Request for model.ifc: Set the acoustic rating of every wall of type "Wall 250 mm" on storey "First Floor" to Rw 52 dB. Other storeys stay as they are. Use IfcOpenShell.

First a look at what the model holds.

```python
import ifcopenshell
import ifcopenshell.util.element

model = ifcopenshell.open("model.ifc")
print(model.schema)
storey = next(s for s in model.by_type("IfcBuildingStorey") if s.Name == "First Floor")
walls = [e for e in ifcopenshell.util.element.get_decomposition(storey) if e.is_a("IfcWall")]
seen = {}
for e in walls:
    element_type = ifcopenshell.util.element.get_type(e)
    key = (element_type.Name if element_type != e and element_type else None, ifcopenshell.util.element.get_pset(e, "Pset_WallCommon", "AcousticRating"))
    seen[key] = seen.get(key, 0) + 1
for (name, value), count in sorted(seen.items(), key=str):
    print(count, "x", name, "|", value)
```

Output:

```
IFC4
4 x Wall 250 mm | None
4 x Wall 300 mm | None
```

```python
import ifcopenshell
import ifcopenshell.api.pset
import ifcopenshell.util.element

model = ifcopenshell.open("model.ifc")

storey = next(s for s in model.by_type("IfcBuildingStorey") if s.Name == "First Floor")
walls = [e for e in ifcopenshell.util.element.get_decomposition(storey) if e.is_a("IfcWall")]

count = 0
for e in walls:
    element_type = ifcopenshell.util.element.get_type(e)
    if element_type in (None, e) or element_type.Name != "Wall 250 mm":
        continue
    # add_pset returns the element's existing set when there is one.
    pset = ifcopenshell.api.pset.add_pset(model, product=e, name="Pset_WallCommon")
    ifcopenshell.api.pset.edit_pset(model, pset=pset, properties={"AcousticRating": "Rw 52 dB"})
    count += 1

print(count, "walls updated")

model.write("model_edited.ifc")
```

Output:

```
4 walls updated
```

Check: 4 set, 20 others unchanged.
